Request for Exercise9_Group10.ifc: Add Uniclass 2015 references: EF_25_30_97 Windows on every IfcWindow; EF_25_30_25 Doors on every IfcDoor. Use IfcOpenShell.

First a look at what the model holds.

```python
import ifcopenshell

model = ifcopenshell.open("Exercise9_Group10.ifc")
print(model.schema)
print("classifications:", [c.Name for c in model.by_type("IfcClassification")])
for ifc_class in ("IfcDoor", "IfcRoof", "IfcStair", "IfcWall", "IfcWindow"):
    print(ifc_class, len(model.by_type(ifc_class)))
```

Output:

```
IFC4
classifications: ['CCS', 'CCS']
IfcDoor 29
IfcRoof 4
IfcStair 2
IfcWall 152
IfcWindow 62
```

```python
import ifcopenshell
import ifcopenshell.api.classification

model = ifcopenshell.open("Exercise9_Group10.ifc")

system = ifcopenshell.api.classification.add_classification(model, classification="Uniclass 2015")

codes = {
    "IfcWindow": ("EF_25_30_97", "Windows"),
    "IfcDoor": ("EF_25_30_25", "Doors"),
}
for ifc_class, (code, name) in codes.items():
    products = model.by_type(ifc_class)
    ifcopenshell.api.classification.add_reference(
        model, products=products, classification=system, identification=code, name=name
    )
    print(code, len(products))

model.write("Exercise9_Group10_v2.ifc")
```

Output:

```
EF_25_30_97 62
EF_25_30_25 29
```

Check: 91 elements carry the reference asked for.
